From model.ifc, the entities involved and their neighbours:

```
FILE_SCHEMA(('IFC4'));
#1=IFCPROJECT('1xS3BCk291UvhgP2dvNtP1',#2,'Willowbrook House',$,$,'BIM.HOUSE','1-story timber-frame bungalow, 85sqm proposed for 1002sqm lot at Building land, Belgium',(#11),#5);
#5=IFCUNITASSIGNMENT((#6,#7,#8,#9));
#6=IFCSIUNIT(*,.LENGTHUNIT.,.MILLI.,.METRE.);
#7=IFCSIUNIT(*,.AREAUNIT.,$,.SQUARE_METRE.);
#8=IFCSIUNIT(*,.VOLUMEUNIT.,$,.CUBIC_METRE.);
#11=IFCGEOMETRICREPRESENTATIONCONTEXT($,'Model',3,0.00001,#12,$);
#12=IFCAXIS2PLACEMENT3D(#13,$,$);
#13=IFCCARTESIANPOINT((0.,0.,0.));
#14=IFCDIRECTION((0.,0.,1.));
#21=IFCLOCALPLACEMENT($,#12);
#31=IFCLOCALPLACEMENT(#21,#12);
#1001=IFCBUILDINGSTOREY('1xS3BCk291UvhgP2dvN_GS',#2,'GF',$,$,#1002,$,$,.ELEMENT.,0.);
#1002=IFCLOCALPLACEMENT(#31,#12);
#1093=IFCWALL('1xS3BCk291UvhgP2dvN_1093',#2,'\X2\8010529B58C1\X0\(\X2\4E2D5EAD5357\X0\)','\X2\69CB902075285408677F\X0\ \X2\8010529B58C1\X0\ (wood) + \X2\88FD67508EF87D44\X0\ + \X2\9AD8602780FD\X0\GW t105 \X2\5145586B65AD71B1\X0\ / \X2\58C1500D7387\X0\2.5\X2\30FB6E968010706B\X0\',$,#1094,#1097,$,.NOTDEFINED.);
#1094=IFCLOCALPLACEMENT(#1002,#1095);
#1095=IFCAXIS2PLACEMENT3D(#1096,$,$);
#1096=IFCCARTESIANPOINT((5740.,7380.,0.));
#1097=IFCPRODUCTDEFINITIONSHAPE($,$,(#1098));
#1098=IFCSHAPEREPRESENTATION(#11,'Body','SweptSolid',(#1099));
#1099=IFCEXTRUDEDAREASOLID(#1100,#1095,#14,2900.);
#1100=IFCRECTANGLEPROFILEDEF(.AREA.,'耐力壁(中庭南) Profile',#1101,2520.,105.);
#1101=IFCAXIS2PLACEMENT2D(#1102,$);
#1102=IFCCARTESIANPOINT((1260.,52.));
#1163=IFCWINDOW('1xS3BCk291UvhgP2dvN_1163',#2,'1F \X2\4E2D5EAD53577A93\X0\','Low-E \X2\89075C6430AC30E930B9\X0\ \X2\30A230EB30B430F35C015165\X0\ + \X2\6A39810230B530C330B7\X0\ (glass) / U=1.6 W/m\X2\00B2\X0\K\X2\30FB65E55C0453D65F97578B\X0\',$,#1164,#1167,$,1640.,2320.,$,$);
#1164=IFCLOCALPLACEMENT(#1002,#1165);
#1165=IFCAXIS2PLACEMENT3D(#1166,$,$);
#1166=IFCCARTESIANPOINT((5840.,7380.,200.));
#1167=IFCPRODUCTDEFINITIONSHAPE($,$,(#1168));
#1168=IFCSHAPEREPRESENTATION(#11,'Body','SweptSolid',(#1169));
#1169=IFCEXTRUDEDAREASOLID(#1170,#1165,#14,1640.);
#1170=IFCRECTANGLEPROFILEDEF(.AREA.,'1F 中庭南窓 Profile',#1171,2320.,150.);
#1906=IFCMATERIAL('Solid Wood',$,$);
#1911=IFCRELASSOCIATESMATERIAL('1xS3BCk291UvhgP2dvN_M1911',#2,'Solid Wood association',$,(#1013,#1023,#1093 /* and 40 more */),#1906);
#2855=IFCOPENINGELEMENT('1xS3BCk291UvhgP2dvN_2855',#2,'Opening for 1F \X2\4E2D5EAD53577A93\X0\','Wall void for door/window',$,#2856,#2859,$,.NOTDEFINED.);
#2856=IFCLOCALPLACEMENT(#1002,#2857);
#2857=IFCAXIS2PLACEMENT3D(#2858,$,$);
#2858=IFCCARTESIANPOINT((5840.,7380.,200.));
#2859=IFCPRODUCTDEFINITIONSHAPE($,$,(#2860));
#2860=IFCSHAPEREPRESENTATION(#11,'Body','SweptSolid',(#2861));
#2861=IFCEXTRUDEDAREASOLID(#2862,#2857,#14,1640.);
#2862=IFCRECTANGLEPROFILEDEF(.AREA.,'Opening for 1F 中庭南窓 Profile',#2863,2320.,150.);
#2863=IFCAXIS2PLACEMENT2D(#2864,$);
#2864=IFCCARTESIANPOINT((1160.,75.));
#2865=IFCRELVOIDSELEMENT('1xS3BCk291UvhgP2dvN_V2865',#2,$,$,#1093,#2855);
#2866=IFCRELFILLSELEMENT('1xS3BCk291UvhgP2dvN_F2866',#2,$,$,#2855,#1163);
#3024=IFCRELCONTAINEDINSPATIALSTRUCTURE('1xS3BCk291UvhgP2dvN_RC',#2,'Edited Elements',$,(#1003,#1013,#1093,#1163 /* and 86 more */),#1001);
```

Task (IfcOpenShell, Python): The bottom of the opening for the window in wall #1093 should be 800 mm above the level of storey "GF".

```python
import numpy as np
import ifcopenshell
import ifcopenshell.api.geometry
import ifcopenshell.geom
import ifcopenshell.util.element
import ifcopenshell.util.placement
import ifcopenshell.util.shape
import ifcopenshell.util.unit

model = ifcopenshell.open("model.ifc")
unit_scale = ifcopenshell.util.unit.calculate_unit_scale(model)

window = model.by_guid("1xS3BCk291UvhgP2dvN_1163")
opening = window.FillsVoids[0].RelatingOpeningElement
storey = ifcopenshell.util.element.get_container(window, ifc_class="IfcBuildingStorey")
level = ifcopenshell.util.placement.get_local_placement(storey.ObjectPlacement)[2, 3]

# The opening's origin need not be at the sill, so measure its lowest point.
shape = ifcopenshell.geom.create_shape(ifcopenshell.geom.settings(), opening)
bottom = ifcopenshell.util.shape.get_shape_bottom_elevation(shape, shape.geometry) / unit_scale
dz = level + 800.0 - bottom

shift = np.array([0.0, 0.0, dz])
# The window is not placed relative to its opening, so move both.
for product in (opening, window):
    matrix = ifcopenshell.util.placement.get_local_placement(product.ObjectPlacement)
    matrix[:3, 3] += shift
    ifcopenshell.api.geometry.edit_object_placement(model, product=product, matrix=matrix, is_si=False)

print(f"moved by {dz * unit_scale:+.3f} m")

model.write("model_rev.ifc")
```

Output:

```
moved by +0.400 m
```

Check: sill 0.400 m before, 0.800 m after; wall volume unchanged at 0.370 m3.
